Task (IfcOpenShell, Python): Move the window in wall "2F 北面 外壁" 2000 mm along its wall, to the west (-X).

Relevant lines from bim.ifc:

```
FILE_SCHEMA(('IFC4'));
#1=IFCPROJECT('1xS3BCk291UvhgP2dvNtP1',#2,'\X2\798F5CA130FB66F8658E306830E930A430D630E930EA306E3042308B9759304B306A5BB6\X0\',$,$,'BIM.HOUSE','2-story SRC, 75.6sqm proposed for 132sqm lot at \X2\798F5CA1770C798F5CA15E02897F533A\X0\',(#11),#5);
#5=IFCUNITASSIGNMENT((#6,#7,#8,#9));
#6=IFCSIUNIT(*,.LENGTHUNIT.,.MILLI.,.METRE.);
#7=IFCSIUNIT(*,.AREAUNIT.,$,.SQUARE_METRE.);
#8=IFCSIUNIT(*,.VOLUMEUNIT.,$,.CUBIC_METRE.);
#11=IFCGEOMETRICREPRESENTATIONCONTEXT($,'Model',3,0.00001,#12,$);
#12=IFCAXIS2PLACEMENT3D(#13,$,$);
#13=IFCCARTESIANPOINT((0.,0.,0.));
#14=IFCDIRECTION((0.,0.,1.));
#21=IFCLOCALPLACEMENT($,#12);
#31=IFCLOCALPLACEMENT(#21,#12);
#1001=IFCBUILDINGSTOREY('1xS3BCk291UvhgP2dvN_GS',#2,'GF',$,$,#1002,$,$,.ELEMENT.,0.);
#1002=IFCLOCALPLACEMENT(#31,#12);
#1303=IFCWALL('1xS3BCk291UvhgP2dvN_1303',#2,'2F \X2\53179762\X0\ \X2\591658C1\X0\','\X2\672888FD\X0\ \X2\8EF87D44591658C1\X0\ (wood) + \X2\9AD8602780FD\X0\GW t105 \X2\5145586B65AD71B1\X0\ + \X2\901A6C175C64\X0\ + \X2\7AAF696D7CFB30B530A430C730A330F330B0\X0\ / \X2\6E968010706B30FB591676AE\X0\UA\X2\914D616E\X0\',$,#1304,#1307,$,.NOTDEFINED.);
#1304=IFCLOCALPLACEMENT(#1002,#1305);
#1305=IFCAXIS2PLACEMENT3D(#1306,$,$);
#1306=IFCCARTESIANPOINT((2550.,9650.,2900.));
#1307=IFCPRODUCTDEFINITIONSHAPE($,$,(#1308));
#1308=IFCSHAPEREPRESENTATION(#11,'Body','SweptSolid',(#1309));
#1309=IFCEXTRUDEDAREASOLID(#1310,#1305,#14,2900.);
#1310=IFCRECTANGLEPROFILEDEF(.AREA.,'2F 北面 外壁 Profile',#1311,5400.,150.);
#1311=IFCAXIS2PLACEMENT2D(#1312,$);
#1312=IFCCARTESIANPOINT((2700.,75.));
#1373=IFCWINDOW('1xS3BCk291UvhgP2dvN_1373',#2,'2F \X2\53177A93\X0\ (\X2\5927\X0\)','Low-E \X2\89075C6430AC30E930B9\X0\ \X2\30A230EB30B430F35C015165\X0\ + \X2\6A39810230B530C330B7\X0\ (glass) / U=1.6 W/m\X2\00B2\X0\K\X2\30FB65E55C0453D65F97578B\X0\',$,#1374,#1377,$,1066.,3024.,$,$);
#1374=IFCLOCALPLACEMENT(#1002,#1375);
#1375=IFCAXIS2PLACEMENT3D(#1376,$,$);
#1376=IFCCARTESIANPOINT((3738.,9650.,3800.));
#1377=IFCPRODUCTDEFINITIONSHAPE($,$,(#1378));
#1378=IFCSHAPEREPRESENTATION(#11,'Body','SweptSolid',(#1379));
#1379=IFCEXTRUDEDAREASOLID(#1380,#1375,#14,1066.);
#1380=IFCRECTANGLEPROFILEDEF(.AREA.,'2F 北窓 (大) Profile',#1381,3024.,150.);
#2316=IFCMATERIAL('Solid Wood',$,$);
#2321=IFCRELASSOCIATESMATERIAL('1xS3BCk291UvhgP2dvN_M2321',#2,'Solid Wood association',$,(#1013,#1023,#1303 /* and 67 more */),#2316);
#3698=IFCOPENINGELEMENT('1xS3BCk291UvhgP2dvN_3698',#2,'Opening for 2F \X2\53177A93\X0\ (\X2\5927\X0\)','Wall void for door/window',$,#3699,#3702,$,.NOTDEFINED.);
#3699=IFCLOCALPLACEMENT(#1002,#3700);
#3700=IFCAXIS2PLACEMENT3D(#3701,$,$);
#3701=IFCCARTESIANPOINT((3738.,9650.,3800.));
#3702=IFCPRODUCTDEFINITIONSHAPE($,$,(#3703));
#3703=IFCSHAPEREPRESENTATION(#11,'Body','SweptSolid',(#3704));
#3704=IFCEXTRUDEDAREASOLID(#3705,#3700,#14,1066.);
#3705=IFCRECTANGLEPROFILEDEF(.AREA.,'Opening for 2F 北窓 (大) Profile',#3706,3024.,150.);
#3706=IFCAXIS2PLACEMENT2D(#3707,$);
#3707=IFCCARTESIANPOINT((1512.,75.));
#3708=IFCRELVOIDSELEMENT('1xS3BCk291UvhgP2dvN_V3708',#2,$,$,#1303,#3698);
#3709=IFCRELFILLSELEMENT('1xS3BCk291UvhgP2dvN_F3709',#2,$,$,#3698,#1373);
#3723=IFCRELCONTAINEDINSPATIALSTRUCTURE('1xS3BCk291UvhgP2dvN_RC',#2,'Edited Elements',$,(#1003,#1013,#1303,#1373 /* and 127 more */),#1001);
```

```python
import ifcopenshell
import ifcopenshell.api.geometry
import ifcopenshell.util.placement

model = ifcopenshell.open("bim.ifc")

window = model.by_id(1373)
opening = window.FillsVoids[0].RelatingOpeningElement
wall = opening.VoidsElements[0].RelatingBuildingElement

wall_matrix = ifcopenshell.util.placement.get_local_placement(wall.ObjectPlacement)
shift = wall_matrix[:3, 0] * -2000.0
before = ifcopenshell.util.placement.get_local_placement(window.ObjectPlacement)[:3, 3].copy()

# The window is not placed relative to its opening, so move both.
for product in (opening, window):
    matrix = ifcopenshell.util.placement.get_local_placement(product.ObjectPlacement)
    matrix[:3, 3] += shift
    ifcopenshell.api.geometry.edit_object_placement(model, product=product, matrix=matrix, is_si=False)

after = ifcopenshell.util.placement.get_local_placement(window.ObjectPlacement)[:3, 3]
print("window moved by", (after - before).round(3) + 0.0)

model.write("bim_edited.ifc")
```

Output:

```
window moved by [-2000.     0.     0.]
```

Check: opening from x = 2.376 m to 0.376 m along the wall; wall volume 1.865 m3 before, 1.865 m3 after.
